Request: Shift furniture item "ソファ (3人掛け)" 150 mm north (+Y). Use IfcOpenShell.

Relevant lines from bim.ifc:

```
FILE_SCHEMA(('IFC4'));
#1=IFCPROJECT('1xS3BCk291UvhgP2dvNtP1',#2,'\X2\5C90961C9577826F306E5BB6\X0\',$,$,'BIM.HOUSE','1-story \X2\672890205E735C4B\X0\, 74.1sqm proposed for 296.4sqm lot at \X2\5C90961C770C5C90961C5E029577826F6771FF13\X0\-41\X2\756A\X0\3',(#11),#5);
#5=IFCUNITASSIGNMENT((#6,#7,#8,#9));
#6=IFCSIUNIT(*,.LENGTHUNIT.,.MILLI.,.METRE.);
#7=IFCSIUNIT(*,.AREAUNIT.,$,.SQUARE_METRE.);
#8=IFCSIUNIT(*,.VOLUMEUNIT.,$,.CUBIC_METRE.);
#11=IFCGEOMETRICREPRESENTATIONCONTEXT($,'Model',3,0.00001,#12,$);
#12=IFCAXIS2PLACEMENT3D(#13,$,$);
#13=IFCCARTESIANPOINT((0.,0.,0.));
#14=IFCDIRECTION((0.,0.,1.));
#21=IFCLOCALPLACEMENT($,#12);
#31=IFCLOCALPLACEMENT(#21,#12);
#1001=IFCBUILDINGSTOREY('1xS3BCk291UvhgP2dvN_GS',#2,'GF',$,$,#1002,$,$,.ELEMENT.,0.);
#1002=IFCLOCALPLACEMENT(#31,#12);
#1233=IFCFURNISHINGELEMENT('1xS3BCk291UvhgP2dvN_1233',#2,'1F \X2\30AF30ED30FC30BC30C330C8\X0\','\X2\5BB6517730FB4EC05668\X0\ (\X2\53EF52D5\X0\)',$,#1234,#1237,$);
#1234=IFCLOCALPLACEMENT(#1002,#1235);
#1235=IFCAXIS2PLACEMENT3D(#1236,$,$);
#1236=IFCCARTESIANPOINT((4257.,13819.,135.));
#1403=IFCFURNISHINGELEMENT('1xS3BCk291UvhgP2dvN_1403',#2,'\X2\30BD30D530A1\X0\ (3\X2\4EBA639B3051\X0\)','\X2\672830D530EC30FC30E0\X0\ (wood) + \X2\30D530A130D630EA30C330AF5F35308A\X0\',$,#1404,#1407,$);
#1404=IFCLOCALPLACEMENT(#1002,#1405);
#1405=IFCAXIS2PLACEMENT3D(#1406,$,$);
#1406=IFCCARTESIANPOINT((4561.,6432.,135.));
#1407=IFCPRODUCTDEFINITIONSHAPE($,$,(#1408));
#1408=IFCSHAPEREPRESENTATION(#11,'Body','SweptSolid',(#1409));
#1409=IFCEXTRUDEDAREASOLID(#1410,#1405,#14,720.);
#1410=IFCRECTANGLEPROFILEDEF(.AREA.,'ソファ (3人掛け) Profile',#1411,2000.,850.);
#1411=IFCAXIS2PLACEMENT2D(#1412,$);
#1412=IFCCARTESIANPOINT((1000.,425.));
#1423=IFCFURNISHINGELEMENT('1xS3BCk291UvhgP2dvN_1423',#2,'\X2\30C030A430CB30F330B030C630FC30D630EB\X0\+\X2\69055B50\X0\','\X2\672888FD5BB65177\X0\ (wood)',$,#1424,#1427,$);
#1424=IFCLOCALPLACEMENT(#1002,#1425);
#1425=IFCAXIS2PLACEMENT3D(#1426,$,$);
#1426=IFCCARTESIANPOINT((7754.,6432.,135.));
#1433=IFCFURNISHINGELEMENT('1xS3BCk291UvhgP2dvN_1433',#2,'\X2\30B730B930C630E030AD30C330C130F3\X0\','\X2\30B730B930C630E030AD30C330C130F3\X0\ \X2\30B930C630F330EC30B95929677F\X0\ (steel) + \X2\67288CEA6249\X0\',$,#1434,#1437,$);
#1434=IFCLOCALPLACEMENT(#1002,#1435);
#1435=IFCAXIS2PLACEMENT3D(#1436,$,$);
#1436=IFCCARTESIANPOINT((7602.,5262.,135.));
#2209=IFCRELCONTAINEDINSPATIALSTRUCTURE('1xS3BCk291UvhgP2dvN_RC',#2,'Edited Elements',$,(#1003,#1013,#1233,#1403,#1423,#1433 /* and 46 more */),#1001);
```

```python
import ifcopenshell
import ifcopenshell.api.geometry
import ifcopenshell.util.placement
import ifcopenshell.util.unit

model = ifcopenshell.open("bim.ifc")
unit_scale = ifcopenshell.util.unit.calculate_unit_scale(model)

item = model.by_guid("1xS3BCk291UvhgP2dvN_1403")
matrix = ifcopenshell.util.placement.get_local_placement(item.ObjectPlacement)
matrix[1, 3] += 0.15 / unit_scale
ifcopenshell.api.geometry.edit_object_placement(model, product=item, matrix=matrix, is_si=False)

print(ifcopenshell.util.placement.get_local_placement(item.ObjectPlacement).round(3) + 0.0)

model.write("bim_rev.ifc")
```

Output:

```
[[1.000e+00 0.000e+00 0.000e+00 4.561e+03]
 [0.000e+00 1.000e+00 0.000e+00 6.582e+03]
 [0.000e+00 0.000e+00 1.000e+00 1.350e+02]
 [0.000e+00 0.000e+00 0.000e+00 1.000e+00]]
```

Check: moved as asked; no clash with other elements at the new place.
